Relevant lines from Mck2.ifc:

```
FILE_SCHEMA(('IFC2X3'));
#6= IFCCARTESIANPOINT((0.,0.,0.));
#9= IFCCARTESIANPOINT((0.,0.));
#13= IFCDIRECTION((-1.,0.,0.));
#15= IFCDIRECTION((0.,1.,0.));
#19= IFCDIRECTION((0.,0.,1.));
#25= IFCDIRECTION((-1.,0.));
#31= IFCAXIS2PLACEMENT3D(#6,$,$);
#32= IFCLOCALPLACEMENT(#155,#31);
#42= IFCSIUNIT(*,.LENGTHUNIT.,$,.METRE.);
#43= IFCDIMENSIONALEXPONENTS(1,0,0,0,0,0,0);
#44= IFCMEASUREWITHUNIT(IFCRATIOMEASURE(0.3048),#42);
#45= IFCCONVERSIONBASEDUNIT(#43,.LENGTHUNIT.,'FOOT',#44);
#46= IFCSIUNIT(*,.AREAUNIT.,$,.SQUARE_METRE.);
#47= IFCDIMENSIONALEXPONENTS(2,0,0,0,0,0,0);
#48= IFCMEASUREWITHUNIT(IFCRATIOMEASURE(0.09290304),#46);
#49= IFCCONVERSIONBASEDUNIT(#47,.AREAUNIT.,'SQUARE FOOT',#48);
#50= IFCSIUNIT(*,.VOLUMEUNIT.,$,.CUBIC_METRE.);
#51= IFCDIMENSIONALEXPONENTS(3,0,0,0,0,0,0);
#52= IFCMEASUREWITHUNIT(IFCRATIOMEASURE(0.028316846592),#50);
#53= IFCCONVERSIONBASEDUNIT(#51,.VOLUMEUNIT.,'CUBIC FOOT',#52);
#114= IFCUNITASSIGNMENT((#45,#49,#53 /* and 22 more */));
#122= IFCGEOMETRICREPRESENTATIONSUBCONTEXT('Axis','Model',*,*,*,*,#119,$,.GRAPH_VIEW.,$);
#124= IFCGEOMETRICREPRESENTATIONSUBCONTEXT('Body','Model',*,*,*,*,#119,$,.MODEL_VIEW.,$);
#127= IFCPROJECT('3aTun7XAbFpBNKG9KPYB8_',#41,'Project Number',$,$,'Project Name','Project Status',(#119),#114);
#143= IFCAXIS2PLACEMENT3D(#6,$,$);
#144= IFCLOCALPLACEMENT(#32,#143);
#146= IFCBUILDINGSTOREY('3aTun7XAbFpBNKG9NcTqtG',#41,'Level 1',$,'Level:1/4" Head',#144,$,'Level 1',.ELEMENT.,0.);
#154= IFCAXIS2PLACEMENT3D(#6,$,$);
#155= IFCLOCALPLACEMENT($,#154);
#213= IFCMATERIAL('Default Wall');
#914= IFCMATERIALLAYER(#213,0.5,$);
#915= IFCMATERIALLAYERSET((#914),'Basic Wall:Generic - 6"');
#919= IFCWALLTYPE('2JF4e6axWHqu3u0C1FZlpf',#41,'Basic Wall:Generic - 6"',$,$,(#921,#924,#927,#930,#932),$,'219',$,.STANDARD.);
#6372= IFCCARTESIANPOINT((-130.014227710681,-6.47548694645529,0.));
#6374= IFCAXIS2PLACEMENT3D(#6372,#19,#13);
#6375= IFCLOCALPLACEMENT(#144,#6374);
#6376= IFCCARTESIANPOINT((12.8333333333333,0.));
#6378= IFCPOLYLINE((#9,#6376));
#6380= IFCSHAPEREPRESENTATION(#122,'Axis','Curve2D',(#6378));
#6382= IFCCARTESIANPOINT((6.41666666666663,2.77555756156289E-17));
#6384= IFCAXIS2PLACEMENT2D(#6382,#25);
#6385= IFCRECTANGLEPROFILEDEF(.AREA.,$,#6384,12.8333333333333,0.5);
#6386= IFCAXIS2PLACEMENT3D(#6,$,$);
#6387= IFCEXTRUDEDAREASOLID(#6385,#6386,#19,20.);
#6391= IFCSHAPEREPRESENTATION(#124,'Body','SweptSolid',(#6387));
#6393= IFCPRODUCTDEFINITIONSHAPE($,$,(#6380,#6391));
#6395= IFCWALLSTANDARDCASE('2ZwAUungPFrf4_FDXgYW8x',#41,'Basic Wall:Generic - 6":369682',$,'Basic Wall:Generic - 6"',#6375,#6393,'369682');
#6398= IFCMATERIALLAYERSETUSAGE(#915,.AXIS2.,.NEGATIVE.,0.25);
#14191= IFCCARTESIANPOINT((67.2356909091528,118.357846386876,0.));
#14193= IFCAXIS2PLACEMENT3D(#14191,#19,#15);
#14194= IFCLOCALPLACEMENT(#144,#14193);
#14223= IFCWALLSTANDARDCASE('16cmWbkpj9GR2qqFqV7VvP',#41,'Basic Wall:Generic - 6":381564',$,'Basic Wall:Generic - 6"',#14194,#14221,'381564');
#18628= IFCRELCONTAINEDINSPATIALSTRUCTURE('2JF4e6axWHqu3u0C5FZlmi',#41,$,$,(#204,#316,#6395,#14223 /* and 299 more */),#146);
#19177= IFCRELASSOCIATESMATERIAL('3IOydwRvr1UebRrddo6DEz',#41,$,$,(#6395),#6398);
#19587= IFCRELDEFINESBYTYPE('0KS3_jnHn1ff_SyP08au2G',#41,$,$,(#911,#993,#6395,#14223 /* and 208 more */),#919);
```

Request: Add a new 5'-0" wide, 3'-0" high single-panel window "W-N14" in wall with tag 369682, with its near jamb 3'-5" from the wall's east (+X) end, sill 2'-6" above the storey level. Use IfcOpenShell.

```python
import numpy as np
import ifcopenshell
import ifcopenshell.api.feature
import ifcopenshell.api.geometry
import ifcopenshell.api.root
import ifcopenshell.api.spatial
import ifcopenshell.api.type
import ifcopenshell.geom
import ifcopenshell.util.element
import ifcopenshell.util.placement
import ifcopenshell.util.representation
import ifcopenshell.util.shape
import ifcopenshell.util.unit

model = ifcopenshell.open("Mck2.ifc")
unit_scale = ifcopenshell.util.unit.calculate_unit_scale(model)
settings = ifcopenshell.geom.settings()


def volume(element):
    """Net volume in cubic metres, openings subtracted."""
    shape = ifcopenshell.geom.create_shape(settings, element)
    return ifcopenshell.util.shape.get_volume(shape.geometry)


wall = model.by_guid("2ZwAUungPFrf4_FDXgYW8x")
storey = ifcopenshell.util.element.get_container(wall, ifc_class="IfcBuildingStorey")
context = ifcopenshell.util.representation.get_context(model, "Model", "Body", "MODEL_VIEW")
before = volume(wall)

width, height, from_end, sill = 1.524, 0.9144, 1.0414, 0.762  # metres

# The wall runs along its own X axis, and the end named is its -X end.
wall_shape = ifcopenshell.geom.create_shape(settings, wall)
x, y, z = ifcopenshell.util.shape.get_vertices(wall_shape.geometry).T
start = x.min() + from_end
face, thickness = float(y.min()), float(y.max() - y.min())
wall_matrix = ifcopenshell.util.placement.get_local_placement(wall.ObjectPlacement)
level = ifcopenshell.util.placement.get_local_placement(storey.ObjectPlacement)[2, 3]


def in_wall(x, y):
    """Placement at x, y metres in the wall's axes, at sill height."""
    matrix = wall_matrix.copy()
    matrix[:, 3] = wall_matrix @ np.array([x / unit_scale, y / unit_scale, 0.0, 1.0])
    matrix[2, 3] = level + sill / unit_scale
    return matrix


# Opening: a box that overshoots both wall faces by 50 mm.
opening = ifcopenshell.api.root.create_entity(model, ifc_class="IfcOpeningElement")
box = ifcopenshell.api.geometry.add_wall_representation(
    model, context=context, length=width, height=height, thickness=thickness + 0.1
)
ifcopenshell.api.geometry.assign_representation(model, product=opening, representation=box)
ifcopenshell.api.geometry.edit_object_placement(model, product=opening, matrix=in_wall(start, face - 0.05), is_si=False)
ifcopenshell.api.feature.add_feature(model, feature=opening, element=wall)

window = ifcopenshell.api.root.create_entity(model, ifc_class="IfcWindow", name="W-N14")
window.OverallWidth, window.OverallHeight = width / unit_scale, height / unit_scale
body = ifcopenshell.api.geometry.add_window_representation(
    model,
    context=context,
    overall_width=window.OverallWidth,
    overall_height=window.OverallHeight,
    partition_type="SINGLE_PANEL",
)
ifcopenshell.api.geometry.assign_representation(model, product=window, representation=body)
ifcopenshell.api.spatial.assign_container(model, products=[window], relating_structure=storey)
fills = ifcopenshell.api.feature.add_filling(model, opening=opening, element=window)
fills.OwnerHistory = window.OwnerHistory  # required in IFC2X3

# IFC2X3 keeps the operation on the window style.
style = ifcopenshell.api.root.create_entity(model, ifc_class="IfcWindowStyle", name="W-N14")
style.OperationType, style.ConstructionType = "SINGLE_PANEL", "NOTDEFINED"
style.ParameterTakesPrecedence = style.Sizeable = False
ifcopenshell.api.type.assign_type(model, related_objects=[window], relating_type=style)

# Centre the window in the wall's thickness.
ifcopenshell.api.geometry.edit_object_placement(model, product=window, matrix=in_wall(start, face), is_si=False)
window_shape = ifcopenshell.geom.create_shape(settings, window)
depth = ifcopenshell.util.shape.get_vertices(window_shape.geometry)[:, 1]
offset = face + thickness / 2 - (depth.min() + depth.max()) / 2
ifcopenshell.api.geometry.edit_object_placement(model, product=window, matrix=in_wall(start, offset), is_si=False)

after = volume(wall)

print(f"wall volume {before:.3f} -> {after:.3f} m3")

model.write("Mck2_rev.ifc")
```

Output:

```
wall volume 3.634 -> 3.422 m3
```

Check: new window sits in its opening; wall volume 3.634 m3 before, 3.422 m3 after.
